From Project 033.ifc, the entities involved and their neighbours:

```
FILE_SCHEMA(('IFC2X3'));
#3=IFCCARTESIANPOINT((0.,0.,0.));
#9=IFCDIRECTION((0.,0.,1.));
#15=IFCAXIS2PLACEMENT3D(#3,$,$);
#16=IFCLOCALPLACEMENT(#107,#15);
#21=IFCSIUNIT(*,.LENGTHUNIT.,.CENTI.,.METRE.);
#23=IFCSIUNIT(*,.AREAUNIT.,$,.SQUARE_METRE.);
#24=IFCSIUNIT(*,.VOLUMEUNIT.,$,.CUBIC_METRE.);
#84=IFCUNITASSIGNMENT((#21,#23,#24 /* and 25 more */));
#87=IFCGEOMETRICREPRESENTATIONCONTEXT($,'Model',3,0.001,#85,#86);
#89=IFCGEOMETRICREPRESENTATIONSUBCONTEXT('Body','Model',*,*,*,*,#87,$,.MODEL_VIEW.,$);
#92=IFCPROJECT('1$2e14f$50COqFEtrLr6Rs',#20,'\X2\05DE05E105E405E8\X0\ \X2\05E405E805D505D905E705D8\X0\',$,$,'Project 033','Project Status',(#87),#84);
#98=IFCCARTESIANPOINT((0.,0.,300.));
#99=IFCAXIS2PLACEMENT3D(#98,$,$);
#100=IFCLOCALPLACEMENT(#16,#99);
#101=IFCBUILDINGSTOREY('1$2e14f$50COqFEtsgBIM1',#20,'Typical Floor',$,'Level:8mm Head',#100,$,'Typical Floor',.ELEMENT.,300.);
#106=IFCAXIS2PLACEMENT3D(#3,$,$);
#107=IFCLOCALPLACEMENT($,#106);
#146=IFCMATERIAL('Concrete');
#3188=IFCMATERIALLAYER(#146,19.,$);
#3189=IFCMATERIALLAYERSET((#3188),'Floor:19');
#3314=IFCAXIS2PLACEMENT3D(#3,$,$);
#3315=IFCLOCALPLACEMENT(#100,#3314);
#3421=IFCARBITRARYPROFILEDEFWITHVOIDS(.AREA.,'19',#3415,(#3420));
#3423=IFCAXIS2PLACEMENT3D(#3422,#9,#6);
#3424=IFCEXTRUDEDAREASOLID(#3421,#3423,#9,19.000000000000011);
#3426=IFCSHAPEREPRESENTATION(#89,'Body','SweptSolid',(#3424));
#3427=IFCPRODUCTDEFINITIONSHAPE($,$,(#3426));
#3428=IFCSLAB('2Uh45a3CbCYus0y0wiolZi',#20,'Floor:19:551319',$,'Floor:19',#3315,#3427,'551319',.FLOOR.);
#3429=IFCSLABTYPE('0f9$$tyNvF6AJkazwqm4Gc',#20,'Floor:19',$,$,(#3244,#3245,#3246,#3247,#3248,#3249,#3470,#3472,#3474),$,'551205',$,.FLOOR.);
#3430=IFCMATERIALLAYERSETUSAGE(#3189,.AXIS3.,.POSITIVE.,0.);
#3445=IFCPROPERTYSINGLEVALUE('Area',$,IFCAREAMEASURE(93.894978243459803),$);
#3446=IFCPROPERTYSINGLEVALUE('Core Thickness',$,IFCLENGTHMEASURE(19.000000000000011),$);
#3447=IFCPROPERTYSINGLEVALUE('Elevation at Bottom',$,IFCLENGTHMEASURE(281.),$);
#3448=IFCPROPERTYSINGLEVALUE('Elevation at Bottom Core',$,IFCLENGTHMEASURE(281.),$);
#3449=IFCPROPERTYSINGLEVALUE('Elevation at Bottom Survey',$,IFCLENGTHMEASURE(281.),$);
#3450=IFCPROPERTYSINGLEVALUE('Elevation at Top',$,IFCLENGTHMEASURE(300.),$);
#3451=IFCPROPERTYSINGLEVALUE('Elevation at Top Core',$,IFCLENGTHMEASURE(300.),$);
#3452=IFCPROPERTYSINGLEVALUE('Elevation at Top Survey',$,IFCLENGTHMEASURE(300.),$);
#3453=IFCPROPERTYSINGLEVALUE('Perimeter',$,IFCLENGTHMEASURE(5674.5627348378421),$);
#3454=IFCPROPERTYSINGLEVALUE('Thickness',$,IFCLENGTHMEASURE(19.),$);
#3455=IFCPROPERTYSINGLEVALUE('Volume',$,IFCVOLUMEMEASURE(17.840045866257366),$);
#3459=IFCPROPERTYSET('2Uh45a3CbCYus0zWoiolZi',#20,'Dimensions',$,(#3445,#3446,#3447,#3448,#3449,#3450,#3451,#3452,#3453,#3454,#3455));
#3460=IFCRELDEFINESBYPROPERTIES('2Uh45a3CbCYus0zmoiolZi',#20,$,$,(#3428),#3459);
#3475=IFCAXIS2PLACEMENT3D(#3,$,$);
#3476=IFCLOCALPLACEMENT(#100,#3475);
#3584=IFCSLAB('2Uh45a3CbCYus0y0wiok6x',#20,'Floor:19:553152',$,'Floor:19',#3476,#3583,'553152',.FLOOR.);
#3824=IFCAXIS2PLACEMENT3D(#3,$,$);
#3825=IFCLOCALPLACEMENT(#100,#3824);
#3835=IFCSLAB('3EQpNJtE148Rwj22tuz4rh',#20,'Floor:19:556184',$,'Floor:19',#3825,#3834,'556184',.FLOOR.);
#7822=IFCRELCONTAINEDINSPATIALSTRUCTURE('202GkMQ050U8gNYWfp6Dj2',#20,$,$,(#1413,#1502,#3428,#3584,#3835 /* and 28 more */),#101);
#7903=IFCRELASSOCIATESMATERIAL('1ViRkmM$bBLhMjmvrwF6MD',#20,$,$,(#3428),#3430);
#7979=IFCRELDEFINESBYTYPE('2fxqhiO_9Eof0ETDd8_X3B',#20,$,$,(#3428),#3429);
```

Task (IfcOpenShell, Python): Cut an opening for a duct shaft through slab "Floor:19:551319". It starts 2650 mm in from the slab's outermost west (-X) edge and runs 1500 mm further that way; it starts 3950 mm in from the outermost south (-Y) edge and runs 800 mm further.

```python
import numpy as np
import ifcopenshell
import ifcopenshell.api.feature
import ifcopenshell.api.geometry
import ifcopenshell.api.pset
import ifcopenshell.api.root
import ifcopenshell.geom
import ifcopenshell.util.element
import ifcopenshell.util.placement
import ifcopenshell.util.representation
import ifcopenshell.util.shape
import ifcopenshell.util.unit

model = ifcopenshell.open("Project 033.ifc")
unit_scale = ifcopenshell.util.unit.calculate_unit_scale(model)
area_scale = ifcopenshell.util.unit.calculate_unit_scale(model, "AREAUNIT")
volume_scale = ifcopenshell.util.unit.calculate_unit_scale(model, "VOLUMEUNIT")
settings = ifcopenshell.geom.settings()


def volume(element):
    """Net volume in cubic metres, openings subtracted."""
    shape = ifcopenshell.geom.create_shape(settings, element)
    return ifcopenshell.util.shape.get_volume(shape.geometry)


slab = model.by_guid("2Uh45a3CbCYus0y0wiolZi")
before = volume(slab)

# Extent in the slab's own axes, in metres. The edges named are its -X and -Y sides.
slab_shape = ifcopenshell.geom.create_shape(settings, slab)
vertices = ifcopenshell.util.shape.get_vertices(slab_shape.geometry)
x_min, y_min, bottom = vertices.min(axis=0)
top = vertices[:, 2].max()

opening = ifcopenshell.api.root.create_entity(model, ifc_class="IfcOpeningElement", name="Duct shaft opening")
context = ifcopenshell.util.representation.get_context(model, "Model", "Body", "MODEL_VIEW")
width, depth = 1.5, 0.8
outline = [(0.0, 0.0), (width, 0.0), (width, depth), (0.0, depth), (0.0, 0.0)]
# Overshoot both faces by 50 mm so the cut is clean.
shape = ifcopenshell.api.geometry.add_slab_representation(
    model, context=context, depth=top - bottom + 0.1, polyline=outline
)
ifcopenshell.api.geometry.assign_representation(model, product=opening, representation=shape)

matrix = ifcopenshell.util.placement.get_local_placement(slab.ObjectPlacement)
matrix[:, 3] = matrix @ np.append(np.array([x_min + 2.65, y_min + 3.95, bottom - 0.05]) / unit_scale, 1.0)
ifcopenshell.api.geometry.edit_object_placement(model, product=opening, matrix=matrix, is_si=False)
ifcopenshell.api.feature.add_feature(model, feature=opening, element=slab)

after = volume(slab)

# Update the slab's stored quantities.
pset = model.by_id(ifcopenshell.util.element.get_pset(slab, "Dimensions", should_inherit=False)["id"])
ifcopenshell.api.pset.edit_pset(model, pset=pset, properties={
    "Area": model.create_entity("IfcAreaMeasure", after / (top - bottom) / area_scale),
    "Volume": model.create_entity("IfcVolumeMeasure", after / volume_scale),
})

print(f"slab volume {before:.3f} -> {after:.3f} m3")

model.write("Project 033_v2.ifc")
```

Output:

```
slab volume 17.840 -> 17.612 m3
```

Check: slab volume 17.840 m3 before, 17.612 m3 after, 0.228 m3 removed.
